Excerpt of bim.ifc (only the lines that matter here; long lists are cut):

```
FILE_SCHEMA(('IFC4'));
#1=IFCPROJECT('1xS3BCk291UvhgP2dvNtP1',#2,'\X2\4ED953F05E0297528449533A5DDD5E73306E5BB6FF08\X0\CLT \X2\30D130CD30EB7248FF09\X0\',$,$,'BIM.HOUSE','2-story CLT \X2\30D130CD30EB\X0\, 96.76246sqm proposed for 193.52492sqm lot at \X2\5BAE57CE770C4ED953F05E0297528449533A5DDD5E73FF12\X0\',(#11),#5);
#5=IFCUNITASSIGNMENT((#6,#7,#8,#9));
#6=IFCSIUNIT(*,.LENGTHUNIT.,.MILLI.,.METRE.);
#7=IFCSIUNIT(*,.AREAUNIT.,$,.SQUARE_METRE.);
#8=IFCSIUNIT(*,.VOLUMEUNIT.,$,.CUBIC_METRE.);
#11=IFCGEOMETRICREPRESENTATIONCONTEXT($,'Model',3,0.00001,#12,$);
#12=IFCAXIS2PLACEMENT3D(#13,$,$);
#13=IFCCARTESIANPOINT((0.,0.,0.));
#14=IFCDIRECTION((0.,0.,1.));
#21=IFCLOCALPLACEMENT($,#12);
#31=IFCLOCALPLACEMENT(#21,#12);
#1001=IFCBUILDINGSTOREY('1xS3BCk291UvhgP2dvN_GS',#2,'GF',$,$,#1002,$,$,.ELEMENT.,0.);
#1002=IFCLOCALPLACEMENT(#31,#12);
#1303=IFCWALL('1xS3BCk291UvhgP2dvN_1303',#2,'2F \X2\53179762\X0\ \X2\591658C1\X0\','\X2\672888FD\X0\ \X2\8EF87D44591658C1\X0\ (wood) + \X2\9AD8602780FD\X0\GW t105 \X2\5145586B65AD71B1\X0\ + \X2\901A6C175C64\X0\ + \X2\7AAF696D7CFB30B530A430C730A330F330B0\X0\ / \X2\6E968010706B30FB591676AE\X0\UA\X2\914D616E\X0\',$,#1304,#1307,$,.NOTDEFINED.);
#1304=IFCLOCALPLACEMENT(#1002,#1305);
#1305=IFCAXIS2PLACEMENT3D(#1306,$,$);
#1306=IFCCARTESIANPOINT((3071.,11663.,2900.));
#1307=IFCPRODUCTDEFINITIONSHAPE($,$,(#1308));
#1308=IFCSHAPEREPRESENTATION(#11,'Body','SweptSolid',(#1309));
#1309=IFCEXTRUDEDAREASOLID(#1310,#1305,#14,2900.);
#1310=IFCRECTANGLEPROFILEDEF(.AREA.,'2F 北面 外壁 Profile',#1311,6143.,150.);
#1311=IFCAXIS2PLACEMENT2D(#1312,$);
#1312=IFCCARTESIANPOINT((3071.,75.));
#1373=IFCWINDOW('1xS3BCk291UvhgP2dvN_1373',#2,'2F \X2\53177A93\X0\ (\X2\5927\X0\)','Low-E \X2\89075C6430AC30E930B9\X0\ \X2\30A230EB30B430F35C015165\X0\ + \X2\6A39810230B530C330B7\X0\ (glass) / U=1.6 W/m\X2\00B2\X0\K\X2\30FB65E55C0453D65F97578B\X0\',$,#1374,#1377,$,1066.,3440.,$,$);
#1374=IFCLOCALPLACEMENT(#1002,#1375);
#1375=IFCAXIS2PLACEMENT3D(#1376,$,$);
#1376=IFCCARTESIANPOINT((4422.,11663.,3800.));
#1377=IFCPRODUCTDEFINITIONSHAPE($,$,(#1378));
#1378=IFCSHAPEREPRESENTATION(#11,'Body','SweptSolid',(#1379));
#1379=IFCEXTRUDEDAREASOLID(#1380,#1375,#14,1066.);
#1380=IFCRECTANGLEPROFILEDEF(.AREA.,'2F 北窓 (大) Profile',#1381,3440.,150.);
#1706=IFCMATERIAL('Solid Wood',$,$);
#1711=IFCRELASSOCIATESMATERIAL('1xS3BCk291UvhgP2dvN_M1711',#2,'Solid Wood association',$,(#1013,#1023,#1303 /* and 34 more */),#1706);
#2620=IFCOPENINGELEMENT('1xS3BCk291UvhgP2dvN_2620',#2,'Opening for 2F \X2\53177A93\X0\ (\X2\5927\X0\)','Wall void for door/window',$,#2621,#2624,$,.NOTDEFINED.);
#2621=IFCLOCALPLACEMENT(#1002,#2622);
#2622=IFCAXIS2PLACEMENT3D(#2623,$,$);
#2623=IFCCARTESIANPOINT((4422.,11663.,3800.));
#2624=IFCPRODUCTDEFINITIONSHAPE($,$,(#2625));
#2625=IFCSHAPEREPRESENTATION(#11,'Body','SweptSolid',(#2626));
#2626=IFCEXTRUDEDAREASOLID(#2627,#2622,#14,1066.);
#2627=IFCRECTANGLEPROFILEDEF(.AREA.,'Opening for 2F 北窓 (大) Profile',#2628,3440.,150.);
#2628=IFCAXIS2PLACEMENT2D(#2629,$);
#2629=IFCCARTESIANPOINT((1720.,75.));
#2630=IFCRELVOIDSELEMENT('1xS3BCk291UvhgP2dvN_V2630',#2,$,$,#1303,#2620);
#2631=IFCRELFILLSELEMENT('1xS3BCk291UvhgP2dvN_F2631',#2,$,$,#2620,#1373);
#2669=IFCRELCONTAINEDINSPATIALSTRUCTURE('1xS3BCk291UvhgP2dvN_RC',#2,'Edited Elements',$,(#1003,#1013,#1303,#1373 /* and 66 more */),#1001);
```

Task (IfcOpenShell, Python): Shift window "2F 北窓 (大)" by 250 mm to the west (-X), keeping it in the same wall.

```python
import ifcopenshell
import ifcopenshell.api.geometry
import ifcopenshell.util.placement
import ifcopenshell.util.unit

model = ifcopenshell.open("bim.ifc")
unit_scale = ifcopenshell.util.unit.calculate_unit_scale(model)

window = model.by_guid("1xS3BCk291UvhgP2dvN_1373")
opening = window.FillsVoids[0].RelatingOpeningElement
wall = opening.VoidsElements[0].RelatingBuildingElement

wall_matrix = ifcopenshell.util.placement.get_local_placement(wall.ObjectPlacement)
shift = wall_matrix[:3, 0] * -0.25 / unit_scale
before = ifcopenshell.util.placement.get_local_placement(window.ObjectPlacement)[:3, 3].copy()

# The window is not placed relative to its opening, so move both.
for product in (opening, window):
    matrix = ifcopenshell.util.placement.get_local_placement(product.ObjectPlacement)
    matrix[:3, 3] += shift
    ifcopenshell.api.geometry.edit_object_placement(model, product=product, matrix=matrix, is_si=False)

after = ifcopenshell.util.placement.get_local_placement(window.ObjectPlacement)[:3, 3]
print("window moved by", (after - before).round(3) + 0.0)

model.write("bim_v2.ifc")
```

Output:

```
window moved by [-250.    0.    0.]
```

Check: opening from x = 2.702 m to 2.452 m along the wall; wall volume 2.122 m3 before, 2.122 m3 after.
